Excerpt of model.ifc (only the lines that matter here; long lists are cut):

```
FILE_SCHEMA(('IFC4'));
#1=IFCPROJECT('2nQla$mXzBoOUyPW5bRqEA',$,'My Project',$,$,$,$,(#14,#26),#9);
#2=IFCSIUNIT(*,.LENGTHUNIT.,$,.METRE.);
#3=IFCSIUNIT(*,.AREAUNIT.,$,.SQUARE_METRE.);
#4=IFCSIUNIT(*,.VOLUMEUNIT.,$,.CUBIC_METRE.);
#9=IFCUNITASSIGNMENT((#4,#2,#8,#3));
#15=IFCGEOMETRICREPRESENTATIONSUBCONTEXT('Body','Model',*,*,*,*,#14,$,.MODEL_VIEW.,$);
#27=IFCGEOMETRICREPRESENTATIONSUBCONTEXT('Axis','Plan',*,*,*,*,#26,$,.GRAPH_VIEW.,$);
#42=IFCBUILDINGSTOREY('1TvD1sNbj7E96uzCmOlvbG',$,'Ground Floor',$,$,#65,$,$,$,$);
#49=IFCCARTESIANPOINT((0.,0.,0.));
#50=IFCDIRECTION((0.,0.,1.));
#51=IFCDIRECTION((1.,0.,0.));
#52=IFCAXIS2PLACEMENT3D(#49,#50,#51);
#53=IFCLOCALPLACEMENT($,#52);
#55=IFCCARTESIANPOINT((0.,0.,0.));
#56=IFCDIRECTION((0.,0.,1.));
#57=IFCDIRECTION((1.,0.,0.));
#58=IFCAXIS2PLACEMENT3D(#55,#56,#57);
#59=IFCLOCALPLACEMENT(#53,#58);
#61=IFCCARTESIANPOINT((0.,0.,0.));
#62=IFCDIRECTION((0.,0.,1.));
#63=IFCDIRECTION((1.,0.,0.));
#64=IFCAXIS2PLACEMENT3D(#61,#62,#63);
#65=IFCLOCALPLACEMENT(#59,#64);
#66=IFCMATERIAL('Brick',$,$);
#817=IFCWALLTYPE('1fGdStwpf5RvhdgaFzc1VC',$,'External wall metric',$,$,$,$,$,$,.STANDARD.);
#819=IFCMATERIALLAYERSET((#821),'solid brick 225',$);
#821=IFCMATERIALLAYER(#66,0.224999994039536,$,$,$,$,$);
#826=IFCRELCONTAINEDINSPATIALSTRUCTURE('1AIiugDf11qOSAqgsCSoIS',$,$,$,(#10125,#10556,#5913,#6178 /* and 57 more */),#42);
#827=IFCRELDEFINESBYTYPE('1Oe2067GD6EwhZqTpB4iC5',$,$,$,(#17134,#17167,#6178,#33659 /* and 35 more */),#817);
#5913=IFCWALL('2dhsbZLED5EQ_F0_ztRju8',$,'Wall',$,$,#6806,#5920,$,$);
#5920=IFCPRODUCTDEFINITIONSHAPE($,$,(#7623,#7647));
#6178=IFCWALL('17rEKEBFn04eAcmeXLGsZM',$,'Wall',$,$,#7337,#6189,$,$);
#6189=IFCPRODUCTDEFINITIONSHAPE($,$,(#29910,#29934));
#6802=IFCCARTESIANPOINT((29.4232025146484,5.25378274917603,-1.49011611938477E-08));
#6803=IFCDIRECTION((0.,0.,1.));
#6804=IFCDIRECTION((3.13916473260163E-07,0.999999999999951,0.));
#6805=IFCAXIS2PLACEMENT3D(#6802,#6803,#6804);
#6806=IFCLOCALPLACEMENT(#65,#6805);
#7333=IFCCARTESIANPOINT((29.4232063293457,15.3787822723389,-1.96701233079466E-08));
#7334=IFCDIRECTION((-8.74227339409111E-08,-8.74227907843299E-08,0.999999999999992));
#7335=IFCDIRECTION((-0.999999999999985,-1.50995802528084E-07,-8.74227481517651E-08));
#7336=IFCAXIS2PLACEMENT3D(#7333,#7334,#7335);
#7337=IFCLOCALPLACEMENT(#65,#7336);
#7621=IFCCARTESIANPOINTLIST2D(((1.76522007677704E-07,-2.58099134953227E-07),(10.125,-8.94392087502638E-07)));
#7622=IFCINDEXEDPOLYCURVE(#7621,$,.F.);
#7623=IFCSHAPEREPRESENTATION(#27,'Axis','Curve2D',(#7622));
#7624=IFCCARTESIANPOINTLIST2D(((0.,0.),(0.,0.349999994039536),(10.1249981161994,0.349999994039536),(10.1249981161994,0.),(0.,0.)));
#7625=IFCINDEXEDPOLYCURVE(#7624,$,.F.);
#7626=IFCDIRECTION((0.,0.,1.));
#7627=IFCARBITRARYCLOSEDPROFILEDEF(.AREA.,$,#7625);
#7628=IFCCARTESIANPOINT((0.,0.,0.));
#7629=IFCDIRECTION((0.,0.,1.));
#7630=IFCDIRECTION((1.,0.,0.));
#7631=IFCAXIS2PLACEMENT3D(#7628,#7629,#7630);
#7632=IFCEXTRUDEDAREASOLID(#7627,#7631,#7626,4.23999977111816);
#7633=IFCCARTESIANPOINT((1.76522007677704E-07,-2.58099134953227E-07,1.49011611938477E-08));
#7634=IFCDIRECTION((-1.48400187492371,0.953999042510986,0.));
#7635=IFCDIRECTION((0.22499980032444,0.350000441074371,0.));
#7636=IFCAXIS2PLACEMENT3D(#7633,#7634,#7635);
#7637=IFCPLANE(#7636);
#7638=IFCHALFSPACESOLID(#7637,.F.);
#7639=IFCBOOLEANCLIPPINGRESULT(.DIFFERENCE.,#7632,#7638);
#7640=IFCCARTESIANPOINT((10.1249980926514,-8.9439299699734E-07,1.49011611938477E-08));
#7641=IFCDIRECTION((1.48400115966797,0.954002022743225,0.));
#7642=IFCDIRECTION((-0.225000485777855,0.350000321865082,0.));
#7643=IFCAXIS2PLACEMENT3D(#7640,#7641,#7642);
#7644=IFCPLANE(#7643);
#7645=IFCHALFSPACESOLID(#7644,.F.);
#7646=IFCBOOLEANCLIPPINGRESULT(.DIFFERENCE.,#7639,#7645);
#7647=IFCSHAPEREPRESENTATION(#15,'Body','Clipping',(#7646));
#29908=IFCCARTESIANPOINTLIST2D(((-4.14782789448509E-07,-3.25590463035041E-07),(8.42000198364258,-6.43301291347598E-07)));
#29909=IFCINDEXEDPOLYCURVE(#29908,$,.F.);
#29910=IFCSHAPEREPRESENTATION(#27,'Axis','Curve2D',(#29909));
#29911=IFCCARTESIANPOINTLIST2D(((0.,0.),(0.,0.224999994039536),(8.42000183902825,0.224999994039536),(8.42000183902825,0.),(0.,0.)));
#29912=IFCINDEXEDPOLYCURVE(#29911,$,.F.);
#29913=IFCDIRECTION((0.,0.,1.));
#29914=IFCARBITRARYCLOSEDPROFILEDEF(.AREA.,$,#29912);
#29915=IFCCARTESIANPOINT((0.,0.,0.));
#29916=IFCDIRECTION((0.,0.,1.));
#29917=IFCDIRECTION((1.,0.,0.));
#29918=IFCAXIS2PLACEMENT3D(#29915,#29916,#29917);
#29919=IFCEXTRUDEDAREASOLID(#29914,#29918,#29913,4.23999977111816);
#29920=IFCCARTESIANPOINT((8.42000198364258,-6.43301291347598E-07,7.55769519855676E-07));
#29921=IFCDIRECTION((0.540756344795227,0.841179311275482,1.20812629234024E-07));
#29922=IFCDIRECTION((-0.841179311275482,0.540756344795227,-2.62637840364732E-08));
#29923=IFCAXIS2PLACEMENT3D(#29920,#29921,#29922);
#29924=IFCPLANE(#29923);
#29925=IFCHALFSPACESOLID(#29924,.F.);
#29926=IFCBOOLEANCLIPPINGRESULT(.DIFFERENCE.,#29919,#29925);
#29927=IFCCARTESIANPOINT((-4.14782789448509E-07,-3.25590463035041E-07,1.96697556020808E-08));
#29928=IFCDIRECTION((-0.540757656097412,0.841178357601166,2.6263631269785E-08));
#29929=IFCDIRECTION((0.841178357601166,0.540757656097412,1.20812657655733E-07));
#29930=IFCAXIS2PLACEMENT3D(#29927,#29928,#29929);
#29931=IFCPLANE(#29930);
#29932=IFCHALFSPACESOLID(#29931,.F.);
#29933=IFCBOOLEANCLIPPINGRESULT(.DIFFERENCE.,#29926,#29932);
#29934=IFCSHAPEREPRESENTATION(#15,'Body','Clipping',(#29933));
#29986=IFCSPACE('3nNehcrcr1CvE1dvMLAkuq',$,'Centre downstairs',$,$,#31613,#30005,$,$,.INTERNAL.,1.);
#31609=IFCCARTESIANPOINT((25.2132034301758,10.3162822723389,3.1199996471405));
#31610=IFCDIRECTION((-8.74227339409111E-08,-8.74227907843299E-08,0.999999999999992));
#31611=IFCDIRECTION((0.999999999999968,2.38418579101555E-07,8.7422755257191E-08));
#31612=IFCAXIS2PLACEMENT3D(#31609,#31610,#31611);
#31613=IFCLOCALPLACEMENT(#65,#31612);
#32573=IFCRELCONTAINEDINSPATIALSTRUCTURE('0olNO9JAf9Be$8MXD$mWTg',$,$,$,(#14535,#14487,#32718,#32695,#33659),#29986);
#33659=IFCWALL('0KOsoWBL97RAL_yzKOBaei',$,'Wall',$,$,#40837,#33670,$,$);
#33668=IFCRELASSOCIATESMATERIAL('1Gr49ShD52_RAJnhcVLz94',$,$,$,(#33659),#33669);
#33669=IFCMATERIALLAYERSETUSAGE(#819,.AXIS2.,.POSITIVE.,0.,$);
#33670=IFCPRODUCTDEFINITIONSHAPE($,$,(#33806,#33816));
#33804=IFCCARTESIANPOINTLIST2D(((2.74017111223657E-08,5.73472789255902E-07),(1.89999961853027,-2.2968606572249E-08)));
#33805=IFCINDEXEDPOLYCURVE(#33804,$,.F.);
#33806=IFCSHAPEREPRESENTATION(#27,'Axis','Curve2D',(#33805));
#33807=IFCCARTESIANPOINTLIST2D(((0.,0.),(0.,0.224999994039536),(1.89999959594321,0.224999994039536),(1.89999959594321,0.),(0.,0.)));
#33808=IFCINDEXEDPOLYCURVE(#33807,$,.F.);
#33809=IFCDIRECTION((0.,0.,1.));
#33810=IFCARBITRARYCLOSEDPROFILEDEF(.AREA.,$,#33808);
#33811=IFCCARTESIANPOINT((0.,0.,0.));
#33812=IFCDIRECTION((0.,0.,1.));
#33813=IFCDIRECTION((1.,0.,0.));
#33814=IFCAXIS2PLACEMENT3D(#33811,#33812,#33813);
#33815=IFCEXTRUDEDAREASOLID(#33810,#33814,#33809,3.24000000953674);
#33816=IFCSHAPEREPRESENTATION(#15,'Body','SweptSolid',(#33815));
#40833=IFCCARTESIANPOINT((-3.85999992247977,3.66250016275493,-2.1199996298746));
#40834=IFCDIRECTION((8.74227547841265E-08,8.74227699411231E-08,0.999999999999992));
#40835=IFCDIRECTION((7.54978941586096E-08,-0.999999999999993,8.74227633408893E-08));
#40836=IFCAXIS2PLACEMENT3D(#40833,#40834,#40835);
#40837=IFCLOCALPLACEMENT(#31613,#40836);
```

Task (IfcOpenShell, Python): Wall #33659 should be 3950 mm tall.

```python
import ifcopenshell
import ifcopenshell.geom
import ifcopenshell.util.representation
import ifcopenshell.util.shape
import ifcopenshell.util.unit

model = ifcopenshell.open("model.ifc")
unit_scale = ifcopenshell.util.unit.calculate_unit_scale(model)
settings = ifcopenshell.geom.settings()


def volume(element):
    """Net volume in cubic metres, openings subtracted."""
    shape = ifcopenshell.geom.create_shape(settings, element)
    return ifcopenshell.util.shape.get_volume(shape.geometry)


wall = model.by_guid("0KOsoWBL97RAL_yzKOBaei")
before = volume(wall)

body = ifcopenshell.util.representation.get_representation(wall, "Model", "Body")
solid = body.Items[0]
old_height = solid.Depth
solid.Depth = 3.95 / unit_scale
after = volume(wall)

print(f"height {old_height:g} -> {solid.Depth:g}, volume {before:.3f} -> {after:.3f} m3")

model.write("model_rev.ifc")
```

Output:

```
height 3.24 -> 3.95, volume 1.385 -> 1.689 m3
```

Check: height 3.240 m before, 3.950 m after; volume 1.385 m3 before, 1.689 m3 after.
